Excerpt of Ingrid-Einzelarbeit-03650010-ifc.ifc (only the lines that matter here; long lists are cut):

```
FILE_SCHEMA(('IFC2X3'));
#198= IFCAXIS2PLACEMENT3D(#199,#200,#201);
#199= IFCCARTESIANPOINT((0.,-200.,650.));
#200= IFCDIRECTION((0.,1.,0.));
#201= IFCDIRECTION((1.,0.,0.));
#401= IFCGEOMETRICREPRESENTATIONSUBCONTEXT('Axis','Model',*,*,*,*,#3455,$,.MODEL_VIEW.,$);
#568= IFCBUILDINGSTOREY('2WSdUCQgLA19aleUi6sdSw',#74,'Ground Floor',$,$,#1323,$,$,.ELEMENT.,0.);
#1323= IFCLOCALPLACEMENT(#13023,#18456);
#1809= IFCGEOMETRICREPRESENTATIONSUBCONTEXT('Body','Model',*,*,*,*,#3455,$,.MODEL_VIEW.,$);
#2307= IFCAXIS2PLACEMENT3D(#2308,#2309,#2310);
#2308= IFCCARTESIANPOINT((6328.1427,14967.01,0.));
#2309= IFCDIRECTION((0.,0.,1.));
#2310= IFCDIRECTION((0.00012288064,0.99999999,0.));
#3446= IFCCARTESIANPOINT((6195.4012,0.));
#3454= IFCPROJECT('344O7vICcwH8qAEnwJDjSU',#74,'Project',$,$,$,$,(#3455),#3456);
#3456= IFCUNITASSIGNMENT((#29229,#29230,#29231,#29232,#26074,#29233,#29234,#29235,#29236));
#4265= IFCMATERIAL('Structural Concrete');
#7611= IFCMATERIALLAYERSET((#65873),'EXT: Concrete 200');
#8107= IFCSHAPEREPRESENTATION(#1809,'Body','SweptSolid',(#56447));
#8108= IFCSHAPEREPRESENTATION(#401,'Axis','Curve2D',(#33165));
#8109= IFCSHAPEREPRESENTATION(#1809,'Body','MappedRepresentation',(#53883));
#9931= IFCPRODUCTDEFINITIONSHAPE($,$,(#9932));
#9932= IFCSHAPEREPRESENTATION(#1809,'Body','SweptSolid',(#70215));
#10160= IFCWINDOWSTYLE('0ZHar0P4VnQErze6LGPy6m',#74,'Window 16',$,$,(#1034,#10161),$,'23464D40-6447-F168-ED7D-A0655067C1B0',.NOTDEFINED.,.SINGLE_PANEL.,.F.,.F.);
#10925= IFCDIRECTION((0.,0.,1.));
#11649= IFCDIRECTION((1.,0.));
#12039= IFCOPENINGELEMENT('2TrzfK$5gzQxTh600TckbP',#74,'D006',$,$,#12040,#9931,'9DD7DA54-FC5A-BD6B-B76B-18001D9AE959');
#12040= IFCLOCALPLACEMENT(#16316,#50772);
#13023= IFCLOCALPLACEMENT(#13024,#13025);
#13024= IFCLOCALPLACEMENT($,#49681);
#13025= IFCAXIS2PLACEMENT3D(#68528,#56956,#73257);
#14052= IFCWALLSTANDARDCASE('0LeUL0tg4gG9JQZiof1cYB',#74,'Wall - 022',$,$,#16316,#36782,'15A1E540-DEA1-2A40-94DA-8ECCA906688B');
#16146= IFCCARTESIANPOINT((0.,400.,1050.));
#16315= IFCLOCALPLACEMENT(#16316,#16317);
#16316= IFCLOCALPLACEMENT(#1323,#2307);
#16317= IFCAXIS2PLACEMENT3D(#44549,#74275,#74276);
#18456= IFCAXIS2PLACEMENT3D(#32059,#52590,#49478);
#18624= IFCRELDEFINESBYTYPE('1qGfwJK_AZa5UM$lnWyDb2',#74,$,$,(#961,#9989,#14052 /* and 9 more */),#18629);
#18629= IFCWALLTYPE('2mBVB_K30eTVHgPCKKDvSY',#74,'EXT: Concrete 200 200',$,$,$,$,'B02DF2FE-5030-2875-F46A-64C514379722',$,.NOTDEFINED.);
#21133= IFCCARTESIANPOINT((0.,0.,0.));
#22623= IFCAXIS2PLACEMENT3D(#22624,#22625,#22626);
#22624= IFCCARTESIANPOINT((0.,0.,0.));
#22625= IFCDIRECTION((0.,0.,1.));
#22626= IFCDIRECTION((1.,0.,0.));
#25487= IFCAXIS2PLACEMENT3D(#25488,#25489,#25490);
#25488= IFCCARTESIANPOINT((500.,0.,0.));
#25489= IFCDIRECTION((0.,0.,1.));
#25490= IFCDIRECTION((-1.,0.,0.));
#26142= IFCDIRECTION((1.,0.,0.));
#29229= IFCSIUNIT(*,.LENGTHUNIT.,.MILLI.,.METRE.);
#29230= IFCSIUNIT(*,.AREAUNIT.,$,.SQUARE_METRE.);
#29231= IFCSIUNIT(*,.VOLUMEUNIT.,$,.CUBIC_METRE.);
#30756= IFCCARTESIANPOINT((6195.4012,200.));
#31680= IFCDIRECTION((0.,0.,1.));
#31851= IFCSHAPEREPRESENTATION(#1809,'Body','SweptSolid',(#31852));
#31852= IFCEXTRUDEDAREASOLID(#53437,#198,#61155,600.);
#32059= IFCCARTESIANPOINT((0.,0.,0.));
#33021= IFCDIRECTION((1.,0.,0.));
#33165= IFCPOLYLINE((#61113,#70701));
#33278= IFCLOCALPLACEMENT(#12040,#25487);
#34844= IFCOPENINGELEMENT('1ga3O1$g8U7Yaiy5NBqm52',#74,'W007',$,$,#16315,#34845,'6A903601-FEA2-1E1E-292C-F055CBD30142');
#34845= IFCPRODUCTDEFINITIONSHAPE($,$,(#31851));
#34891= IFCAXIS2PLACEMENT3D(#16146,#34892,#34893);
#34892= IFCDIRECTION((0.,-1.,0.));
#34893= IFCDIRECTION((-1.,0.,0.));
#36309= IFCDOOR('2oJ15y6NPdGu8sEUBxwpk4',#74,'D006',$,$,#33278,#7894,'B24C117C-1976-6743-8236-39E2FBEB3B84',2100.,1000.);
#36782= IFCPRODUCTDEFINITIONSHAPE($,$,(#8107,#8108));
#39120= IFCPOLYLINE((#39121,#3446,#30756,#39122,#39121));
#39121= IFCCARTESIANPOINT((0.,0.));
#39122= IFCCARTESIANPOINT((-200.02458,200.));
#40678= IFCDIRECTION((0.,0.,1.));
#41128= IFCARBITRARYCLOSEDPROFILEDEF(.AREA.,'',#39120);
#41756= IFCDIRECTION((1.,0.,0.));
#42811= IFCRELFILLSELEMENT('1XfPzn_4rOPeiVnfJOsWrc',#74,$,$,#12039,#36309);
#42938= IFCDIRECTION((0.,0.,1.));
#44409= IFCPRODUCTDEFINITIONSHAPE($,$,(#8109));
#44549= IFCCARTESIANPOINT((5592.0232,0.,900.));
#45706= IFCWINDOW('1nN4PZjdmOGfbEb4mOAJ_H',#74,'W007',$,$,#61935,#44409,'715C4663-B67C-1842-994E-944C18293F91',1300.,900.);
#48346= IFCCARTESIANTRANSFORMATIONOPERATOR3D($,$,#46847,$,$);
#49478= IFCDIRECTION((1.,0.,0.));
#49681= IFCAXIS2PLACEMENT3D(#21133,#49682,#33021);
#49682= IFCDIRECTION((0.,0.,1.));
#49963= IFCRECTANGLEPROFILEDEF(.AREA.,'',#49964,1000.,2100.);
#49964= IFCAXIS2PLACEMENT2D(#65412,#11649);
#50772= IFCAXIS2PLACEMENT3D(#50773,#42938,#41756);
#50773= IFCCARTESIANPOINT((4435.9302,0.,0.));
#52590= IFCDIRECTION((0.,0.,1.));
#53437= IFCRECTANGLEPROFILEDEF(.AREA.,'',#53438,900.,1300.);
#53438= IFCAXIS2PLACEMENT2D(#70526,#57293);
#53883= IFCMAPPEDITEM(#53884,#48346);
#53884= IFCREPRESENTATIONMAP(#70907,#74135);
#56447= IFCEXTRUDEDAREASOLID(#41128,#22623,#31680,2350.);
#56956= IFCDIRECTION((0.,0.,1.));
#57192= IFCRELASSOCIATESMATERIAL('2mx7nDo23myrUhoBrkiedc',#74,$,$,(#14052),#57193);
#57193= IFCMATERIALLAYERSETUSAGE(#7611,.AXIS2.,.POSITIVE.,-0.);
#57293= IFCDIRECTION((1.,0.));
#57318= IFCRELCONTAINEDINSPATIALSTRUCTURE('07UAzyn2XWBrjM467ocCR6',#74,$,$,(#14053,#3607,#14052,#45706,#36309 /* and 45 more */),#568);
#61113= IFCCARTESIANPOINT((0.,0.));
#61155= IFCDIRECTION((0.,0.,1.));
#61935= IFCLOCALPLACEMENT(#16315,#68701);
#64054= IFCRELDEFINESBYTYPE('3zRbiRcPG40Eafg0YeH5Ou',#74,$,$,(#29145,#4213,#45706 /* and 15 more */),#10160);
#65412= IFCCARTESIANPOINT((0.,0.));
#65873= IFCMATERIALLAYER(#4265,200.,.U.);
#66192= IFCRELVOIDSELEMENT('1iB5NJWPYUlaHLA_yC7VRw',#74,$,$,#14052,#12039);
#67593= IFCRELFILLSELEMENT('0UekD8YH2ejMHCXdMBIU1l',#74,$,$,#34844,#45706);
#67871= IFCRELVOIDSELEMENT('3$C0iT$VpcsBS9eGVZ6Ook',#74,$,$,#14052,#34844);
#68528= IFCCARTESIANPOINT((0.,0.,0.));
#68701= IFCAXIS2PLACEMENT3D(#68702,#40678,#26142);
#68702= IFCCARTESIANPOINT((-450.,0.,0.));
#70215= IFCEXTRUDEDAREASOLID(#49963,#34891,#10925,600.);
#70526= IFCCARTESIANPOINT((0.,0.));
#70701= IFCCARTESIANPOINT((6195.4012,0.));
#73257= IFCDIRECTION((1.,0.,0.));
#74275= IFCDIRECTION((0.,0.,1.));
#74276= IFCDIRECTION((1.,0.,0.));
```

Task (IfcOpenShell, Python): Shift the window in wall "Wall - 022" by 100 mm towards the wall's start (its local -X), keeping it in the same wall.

```python
import ifcopenshell
import ifcopenshell.api.geometry
import ifcopenshell.util.placement
import ifcopenshell.util.unit

model = ifcopenshell.open("Ingrid-Einzelarbeit-03650010-ifc.ifc")
unit_scale = ifcopenshell.util.unit.calculate_unit_scale(model)

window = model.by_guid("1nN4PZjdmOGfbEb4mOAJ_H")
opening = window.FillsVoids[0].RelatingOpeningElement
wall = opening.VoidsElements[0].RelatingBuildingElement

wall_matrix = ifcopenshell.util.placement.get_local_placement(wall.ObjectPlacement)
shift = wall_matrix[:3, 0] * -0.1 / unit_scale
before = ifcopenshell.util.placement.get_local_placement(window.ObjectPlacement)[:3, 3].copy()

# The window is placed relative to its opening, so it follows when the opening moves.
matrix = ifcopenshell.util.placement.get_local_placement(opening.ObjectPlacement)
matrix[:3, 3] += shift
ifcopenshell.api.geometry.edit_object_placement(
    model, product=opening, matrix=matrix, is_si=False, should_transform_children=True
)

after = ifcopenshell.util.placement.get_local_placement(window.ObjectPlacement)[:3, 3]
print("window moved by", (after - before).round(3) + 0.0)

model.write("Ingrid-Einzelarbeit-03650010-ifc-out.ifc")
```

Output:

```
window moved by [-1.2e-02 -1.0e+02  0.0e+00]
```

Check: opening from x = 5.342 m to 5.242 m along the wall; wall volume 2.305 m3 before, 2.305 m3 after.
